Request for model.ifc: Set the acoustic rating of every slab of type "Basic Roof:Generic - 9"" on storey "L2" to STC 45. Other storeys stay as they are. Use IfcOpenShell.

First a look at what the model holds.

```python
import ifcopenshell
import ifcopenshell.util.element

model = ifcopenshell.open("model.ifc")
print(model.schema)
storey = next(s for s in model.by_type("IfcBuildingStorey") if s.Name == "L2")
slabs = [e for e in ifcopenshell.util.element.get_decomposition(storey) if e.is_a("IfcSlab")]
seen = {}
for e in slabs:
    element_type = ifcopenshell.util.element.get_type(e)
    key = (element_type.Name if element_type != e and element_type else None, ifcopenshell.util.element.get_pset(e, "Pset_SlabCommon", "AcousticRating"))
    seen[key] = seen.get(key, 0) + 1
for (name, value), count in sorted(seen.items(), key=str):
    print(count, "x", name, "|", value)
```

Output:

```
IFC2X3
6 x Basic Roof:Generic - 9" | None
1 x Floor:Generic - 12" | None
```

```python
import ifcopenshell
import ifcopenshell.api.pset
import ifcopenshell.util.element

model = ifcopenshell.open("model.ifc")

storey = next(s for s in model.by_type("IfcBuildingStorey") if s.Name == "L2")
slabs = [e for e in ifcopenshell.util.element.get_decomposition(storey) if e.is_a("IfcSlab")]

count = 0
for e in slabs:
    element_type = ifcopenshell.util.element.get_type(e)
    if element_type in (None, e) or element_type.Name != 'Basic Roof:Generic - 9"':
        continue
    # add_pset returns the element's existing set when there is one.
    pset = ifcopenshell.api.pset.add_pset(model, product=e, name="Pset_SlabCommon")
    ifcopenshell.api.pset.edit_pset(model, pset=pset, properties={"AcousticRating": "STC 45"})
    count += 1

print(count, "slabs updated")

model.write("model_v2.ifc")
```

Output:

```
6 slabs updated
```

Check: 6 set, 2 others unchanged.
